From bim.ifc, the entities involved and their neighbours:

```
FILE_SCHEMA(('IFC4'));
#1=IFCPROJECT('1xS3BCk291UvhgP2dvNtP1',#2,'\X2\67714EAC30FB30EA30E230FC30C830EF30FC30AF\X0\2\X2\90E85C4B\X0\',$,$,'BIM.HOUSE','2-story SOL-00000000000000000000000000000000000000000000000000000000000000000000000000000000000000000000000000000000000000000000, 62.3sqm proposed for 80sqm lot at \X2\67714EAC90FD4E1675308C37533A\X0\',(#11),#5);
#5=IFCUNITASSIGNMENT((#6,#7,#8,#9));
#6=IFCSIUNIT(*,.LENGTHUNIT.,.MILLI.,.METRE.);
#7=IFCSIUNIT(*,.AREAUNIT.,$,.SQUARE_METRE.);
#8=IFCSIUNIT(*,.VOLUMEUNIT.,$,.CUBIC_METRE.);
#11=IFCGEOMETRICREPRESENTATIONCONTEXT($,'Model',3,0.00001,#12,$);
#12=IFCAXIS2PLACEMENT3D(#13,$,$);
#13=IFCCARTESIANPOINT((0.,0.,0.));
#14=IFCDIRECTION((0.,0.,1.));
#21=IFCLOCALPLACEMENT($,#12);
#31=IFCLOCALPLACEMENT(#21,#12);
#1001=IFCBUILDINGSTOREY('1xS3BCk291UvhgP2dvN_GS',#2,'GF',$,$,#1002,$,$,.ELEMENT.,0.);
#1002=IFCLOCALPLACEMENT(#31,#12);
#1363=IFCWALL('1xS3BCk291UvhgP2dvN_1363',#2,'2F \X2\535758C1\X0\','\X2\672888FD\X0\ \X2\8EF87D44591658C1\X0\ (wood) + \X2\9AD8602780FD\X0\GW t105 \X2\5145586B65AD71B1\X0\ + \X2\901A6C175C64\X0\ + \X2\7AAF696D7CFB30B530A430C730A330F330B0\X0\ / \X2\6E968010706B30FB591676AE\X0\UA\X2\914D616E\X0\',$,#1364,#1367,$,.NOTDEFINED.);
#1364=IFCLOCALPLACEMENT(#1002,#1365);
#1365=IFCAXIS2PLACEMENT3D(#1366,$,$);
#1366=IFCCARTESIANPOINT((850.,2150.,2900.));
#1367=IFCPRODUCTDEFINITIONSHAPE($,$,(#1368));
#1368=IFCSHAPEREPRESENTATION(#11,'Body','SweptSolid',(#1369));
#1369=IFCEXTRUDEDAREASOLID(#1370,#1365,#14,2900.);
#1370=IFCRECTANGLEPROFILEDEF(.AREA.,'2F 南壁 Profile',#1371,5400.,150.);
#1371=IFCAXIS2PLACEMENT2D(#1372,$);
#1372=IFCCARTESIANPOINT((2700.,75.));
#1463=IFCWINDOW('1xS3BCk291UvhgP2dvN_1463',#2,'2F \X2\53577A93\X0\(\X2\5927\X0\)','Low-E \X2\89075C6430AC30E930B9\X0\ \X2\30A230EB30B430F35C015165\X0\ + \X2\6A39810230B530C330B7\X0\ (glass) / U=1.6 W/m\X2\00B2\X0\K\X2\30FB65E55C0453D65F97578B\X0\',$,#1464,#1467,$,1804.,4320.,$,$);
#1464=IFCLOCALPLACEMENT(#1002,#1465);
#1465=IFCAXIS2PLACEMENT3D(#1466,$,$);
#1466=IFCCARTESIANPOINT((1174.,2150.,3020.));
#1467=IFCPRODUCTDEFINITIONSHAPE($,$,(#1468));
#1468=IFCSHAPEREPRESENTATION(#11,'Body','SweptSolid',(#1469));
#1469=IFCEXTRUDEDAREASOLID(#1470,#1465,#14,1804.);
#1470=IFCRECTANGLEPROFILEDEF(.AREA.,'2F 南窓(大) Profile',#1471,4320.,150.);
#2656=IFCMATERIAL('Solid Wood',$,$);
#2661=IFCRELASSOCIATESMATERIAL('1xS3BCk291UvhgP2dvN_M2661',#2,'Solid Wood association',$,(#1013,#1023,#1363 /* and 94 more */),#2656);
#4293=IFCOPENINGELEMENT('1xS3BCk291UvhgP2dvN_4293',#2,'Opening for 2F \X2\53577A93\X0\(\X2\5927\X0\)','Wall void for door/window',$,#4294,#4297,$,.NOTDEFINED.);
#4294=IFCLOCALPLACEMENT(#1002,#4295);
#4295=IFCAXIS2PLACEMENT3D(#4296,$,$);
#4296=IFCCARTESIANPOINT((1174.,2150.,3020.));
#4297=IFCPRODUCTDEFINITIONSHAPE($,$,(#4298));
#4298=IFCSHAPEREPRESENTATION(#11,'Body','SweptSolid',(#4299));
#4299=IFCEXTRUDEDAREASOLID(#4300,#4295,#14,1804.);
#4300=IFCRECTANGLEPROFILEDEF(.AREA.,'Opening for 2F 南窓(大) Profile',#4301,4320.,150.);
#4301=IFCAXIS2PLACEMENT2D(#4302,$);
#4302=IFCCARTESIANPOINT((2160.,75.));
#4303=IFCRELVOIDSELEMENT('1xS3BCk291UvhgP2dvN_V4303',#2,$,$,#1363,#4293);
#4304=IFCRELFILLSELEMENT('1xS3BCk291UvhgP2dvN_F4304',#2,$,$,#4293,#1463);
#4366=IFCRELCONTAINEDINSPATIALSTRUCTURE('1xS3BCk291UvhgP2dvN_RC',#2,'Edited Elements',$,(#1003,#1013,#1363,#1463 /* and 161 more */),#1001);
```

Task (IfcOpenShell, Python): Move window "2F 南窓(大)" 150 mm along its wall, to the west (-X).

```python
import ifcopenshell
import ifcopenshell.api.geometry
import ifcopenshell.util.placement

model = ifcopenshell.open("bim.ifc")

window = model.by_guid("1xS3BCk291UvhgP2dvN_1463")
opening = window.FillsVoids[0].RelatingOpeningElement
wall = opening.VoidsElements[0].RelatingBuildingElement

wall_matrix = ifcopenshell.util.placement.get_local_placement(wall.ObjectPlacement)
shift = wall_matrix[:3, 0] * -150.0
before = ifcopenshell.util.placement.get_local_placement(window.ObjectPlacement)[:3, 3].copy()

# The window is not placed relative to its opening, so move both.
for product in (opening, window):
    matrix = ifcopenshell.util.placement.get_local_placement(product.ObjectPlacement)
    matrix[:3, 3] += shift
    ifcopenshell.api.geometry.edit_object_placement(model, product=product, matrix=matrix, is_si=False)

after = ifcopenshell.util.placement.get_local_placement(window.ObjectPlacement)[:3, 3]
print("window moved by", (after - before).round(3) + 0.0)

model.write("bim_edited.ifc")
```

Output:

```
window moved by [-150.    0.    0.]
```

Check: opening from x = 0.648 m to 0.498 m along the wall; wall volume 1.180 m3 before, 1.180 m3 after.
